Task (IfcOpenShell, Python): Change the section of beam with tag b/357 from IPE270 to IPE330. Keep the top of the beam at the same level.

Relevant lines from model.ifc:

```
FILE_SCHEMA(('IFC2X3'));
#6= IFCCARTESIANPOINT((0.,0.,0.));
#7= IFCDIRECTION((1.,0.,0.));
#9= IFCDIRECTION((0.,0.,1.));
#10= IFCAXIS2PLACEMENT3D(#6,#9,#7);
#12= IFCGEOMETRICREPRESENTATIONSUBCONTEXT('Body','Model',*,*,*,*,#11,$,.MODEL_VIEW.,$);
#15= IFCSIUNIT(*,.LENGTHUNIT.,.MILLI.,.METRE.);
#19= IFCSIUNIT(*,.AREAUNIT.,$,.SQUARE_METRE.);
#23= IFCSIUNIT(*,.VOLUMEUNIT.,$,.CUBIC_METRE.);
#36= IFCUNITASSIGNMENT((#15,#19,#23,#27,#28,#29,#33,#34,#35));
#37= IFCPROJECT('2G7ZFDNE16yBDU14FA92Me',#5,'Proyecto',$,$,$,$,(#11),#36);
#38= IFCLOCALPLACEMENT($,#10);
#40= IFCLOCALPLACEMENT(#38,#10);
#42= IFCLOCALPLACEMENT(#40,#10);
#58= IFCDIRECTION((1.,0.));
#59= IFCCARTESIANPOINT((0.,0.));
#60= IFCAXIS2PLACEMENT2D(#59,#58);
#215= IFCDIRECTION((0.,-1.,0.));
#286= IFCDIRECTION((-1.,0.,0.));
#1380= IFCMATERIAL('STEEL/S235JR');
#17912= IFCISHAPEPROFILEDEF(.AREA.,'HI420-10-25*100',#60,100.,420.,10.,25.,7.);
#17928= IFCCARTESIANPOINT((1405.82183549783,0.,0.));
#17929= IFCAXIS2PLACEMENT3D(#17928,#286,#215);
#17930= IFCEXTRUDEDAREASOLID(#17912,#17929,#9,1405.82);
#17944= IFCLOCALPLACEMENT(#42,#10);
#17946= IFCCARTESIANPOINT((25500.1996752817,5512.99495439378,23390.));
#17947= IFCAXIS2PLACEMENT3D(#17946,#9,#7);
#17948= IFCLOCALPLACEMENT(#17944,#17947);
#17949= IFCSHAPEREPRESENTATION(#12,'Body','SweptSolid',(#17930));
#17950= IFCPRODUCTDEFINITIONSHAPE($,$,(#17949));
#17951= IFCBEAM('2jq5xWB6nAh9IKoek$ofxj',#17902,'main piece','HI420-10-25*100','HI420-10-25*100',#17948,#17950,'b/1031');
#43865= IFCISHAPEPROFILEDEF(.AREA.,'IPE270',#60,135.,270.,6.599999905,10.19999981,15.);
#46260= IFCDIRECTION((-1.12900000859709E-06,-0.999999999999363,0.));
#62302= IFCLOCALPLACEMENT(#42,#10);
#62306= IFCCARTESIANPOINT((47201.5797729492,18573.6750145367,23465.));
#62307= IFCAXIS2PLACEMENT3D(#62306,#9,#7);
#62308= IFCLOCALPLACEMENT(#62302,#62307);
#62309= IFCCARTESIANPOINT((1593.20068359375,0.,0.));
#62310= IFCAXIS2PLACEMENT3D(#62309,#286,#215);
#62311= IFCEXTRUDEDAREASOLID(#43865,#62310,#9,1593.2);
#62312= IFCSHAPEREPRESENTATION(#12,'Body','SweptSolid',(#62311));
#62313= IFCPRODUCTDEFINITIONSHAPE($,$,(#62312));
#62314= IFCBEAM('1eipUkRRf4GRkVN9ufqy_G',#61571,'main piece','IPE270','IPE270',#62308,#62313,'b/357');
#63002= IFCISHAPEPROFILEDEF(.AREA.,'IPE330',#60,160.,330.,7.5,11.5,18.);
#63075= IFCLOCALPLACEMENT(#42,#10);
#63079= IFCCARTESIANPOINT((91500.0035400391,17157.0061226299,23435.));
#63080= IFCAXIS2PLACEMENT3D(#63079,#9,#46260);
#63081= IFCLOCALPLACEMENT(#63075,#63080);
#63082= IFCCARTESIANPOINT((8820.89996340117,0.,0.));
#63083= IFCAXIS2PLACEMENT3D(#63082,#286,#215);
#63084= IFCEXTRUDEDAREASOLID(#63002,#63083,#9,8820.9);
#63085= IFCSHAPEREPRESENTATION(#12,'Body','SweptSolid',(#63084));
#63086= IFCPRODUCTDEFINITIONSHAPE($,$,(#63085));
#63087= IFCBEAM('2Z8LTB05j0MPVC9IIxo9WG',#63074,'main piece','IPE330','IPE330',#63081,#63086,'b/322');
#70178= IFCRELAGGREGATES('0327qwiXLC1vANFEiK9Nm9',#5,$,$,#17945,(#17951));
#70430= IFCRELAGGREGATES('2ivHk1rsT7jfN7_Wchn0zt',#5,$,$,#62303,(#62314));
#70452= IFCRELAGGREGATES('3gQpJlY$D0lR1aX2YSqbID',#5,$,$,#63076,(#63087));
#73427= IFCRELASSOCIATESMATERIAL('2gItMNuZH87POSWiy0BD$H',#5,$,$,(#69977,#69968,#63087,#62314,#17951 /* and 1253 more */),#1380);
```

```python
import ifcopenshell
import ifcopenshell.util.element
import ifcopenshell.util.representation

model = ifcopenshell.open("model.ifc")

member = model.by_id(62314)
source = next(p for p in model.by_type("IfcIShapeProfileDef") if p.ProfileName == "IPE330")

body = ifcopenshell.util.representation.get_representation(member, "Model", "Body")
solid = body.Items[0]
old_profile = solid.SweptArea

# Copy the section's sizes but keep this member's own profile position.
profile = ifcopenshell.util.element.copy(model, source)
# Profiles are centred, so shift by half the change in depth to hold the top.
shift = (old_profile.OverallDepth - profile.OverallDepth) / 2
x, y = old_profile.Position.Location.Coordinates
up = (0.0, 1.0)  # upwards, in the solid's own plane
location = model.createIfcCartesianPoint((x + up[0] * shift, y + up[1] * shift))
profile.Position = model.createIfcAxis2Placement2D(location, old_profile.Position.RefDirection)
solid.SweptArea = profile
if not model.get_total_inverses(old_profile):
    ifcopenshell.util.element.remove_deep2(model, old_profile)
member.Description = member.Description.replace("IPE270", "IPE330")
member.ObjectType = member.ObjectType.replace("IPE270", "IPE330")

print(solid.SweptArea)

model.write("model_updated.ifc")
```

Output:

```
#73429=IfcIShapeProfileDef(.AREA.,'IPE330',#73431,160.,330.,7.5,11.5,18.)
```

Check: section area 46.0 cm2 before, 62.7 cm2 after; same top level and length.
